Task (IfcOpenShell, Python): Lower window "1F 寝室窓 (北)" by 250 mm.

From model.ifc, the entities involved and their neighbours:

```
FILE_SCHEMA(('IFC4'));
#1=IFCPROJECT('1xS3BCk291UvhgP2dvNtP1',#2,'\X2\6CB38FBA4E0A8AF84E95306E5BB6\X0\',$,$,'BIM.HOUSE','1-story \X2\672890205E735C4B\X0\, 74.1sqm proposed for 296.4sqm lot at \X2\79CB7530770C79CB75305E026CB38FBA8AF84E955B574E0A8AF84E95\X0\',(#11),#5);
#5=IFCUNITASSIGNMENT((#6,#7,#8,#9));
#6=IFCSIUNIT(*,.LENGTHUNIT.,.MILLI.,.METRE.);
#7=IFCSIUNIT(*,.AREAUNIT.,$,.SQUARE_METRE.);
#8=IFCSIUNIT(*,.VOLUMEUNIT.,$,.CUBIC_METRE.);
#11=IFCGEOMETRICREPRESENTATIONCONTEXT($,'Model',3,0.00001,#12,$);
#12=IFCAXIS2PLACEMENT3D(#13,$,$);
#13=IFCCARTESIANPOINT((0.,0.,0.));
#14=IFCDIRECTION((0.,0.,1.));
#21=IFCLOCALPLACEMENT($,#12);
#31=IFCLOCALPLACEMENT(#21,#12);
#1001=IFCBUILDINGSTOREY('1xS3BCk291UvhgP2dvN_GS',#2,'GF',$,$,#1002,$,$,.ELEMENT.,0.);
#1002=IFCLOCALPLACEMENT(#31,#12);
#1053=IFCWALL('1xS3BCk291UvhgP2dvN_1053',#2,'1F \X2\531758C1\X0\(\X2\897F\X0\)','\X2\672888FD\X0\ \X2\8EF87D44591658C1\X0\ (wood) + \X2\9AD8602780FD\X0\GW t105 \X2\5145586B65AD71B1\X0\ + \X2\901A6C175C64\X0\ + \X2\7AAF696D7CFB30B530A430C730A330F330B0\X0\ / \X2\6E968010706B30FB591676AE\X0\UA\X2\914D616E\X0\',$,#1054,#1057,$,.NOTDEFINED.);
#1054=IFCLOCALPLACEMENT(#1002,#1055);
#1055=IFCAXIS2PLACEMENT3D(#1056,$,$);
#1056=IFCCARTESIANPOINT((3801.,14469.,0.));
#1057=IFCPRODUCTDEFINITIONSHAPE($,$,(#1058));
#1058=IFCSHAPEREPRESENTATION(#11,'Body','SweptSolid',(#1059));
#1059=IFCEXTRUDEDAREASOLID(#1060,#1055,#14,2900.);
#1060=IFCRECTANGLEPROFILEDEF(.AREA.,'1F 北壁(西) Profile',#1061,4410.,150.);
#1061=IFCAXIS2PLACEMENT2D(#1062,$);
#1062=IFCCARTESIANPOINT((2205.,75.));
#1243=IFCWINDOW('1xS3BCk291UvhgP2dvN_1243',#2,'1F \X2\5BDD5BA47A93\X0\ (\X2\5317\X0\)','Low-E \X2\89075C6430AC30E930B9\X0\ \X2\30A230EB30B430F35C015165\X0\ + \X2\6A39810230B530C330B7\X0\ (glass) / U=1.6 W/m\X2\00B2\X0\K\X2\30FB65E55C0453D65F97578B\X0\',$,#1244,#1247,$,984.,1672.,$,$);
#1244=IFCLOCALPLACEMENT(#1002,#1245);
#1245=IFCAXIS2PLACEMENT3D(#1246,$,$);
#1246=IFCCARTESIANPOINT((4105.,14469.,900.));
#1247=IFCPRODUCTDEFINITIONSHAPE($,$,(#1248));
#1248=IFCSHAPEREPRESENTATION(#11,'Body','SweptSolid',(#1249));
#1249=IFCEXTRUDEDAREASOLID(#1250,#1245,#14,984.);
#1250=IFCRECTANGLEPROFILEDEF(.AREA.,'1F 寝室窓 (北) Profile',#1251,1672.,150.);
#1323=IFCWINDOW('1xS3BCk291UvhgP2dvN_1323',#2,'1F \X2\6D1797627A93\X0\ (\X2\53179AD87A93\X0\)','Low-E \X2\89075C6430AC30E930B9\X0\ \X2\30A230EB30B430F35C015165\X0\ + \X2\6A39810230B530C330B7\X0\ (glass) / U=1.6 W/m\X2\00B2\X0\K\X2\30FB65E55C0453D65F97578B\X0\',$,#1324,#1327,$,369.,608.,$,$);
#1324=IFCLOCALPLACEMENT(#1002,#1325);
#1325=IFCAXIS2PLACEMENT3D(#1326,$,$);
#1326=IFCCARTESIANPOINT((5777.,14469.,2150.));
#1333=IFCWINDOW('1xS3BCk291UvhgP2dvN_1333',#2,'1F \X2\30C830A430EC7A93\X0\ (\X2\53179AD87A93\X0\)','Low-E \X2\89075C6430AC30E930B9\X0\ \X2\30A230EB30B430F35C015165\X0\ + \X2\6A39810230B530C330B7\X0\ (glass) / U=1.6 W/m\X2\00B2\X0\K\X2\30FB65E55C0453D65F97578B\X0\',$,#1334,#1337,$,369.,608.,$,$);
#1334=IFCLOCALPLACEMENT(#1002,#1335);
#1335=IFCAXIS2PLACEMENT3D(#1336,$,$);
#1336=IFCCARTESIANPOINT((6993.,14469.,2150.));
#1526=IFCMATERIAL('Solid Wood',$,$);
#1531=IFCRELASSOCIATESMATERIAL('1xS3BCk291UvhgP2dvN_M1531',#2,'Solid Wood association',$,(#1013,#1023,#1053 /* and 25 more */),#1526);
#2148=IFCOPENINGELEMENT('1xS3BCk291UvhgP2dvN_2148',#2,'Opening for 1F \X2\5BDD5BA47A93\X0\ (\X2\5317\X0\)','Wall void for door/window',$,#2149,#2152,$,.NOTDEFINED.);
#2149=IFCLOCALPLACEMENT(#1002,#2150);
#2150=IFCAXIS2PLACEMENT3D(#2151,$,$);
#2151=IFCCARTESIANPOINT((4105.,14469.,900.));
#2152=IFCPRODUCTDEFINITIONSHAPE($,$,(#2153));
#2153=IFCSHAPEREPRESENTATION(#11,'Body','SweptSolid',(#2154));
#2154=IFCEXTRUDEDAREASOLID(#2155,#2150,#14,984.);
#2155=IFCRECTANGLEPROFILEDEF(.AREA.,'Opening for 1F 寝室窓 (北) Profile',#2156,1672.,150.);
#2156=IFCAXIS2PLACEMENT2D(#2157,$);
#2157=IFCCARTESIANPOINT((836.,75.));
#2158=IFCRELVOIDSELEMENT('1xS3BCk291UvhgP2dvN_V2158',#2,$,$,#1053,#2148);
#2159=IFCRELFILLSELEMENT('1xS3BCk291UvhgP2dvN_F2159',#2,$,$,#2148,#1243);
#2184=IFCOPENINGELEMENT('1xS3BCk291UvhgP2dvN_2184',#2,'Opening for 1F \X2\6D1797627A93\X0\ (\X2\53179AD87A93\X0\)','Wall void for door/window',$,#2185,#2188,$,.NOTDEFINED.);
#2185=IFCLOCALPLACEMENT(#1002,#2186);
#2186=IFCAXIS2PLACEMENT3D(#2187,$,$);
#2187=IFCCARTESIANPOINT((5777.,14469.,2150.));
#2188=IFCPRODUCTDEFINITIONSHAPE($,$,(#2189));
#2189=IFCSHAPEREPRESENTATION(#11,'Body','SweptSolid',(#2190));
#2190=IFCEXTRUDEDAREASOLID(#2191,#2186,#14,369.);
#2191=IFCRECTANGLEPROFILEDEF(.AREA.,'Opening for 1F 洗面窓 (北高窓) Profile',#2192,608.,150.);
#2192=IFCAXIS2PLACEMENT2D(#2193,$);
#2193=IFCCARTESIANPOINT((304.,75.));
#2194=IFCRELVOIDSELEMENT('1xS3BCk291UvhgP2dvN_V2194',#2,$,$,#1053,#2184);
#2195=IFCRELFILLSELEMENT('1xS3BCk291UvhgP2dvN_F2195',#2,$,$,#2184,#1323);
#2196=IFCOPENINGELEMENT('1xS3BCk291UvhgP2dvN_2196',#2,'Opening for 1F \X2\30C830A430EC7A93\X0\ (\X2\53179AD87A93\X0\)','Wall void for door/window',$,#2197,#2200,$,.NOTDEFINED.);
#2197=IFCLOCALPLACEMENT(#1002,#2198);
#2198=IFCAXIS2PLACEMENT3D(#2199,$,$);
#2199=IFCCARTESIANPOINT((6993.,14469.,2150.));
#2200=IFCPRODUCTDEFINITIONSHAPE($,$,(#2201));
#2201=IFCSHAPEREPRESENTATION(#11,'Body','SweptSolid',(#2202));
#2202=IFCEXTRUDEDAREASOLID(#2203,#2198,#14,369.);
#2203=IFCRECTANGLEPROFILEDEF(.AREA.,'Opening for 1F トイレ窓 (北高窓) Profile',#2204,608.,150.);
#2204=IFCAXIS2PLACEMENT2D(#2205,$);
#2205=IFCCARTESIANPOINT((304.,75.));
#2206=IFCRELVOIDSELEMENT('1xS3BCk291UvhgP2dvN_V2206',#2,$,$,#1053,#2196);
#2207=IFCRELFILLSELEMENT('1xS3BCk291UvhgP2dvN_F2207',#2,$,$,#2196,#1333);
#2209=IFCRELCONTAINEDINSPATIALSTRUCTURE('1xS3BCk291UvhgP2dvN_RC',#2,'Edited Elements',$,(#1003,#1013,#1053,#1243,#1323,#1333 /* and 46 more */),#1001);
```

```python
import numpy as np
import ifcopenshell
import ifcopenshell.api.geometry
import ifcopenshell.util.placement
import ifcopenshell.util.unit

model = ifcopenshell.open("model.ifc")
unit_scale = ifcopenshell.util.unit.calculate_unit_scale(model)

window = model.by_guid("1xS3BCk291UvhgP2dvN_1243")
opening = window.FillsVoids[0].RelatingOpeningElement
dz = -250.0

shift = np.array([0.0, 0.0, dz])
# The window is not placed relative to its opening, so move both.
for product in (opening, window):
    matrix = ifcopenshell.util.placement.get_local_placement(product.ObjectPlacement)
    matrix[:3, 3] += shift
    ifcopenshell.api.geometry.edit_object_placement(model, product=product, matrix=matrix, is_si=False)

print(f"moved by {dz * unit_scale:+.3f} m")

model.write("model_edited.ifc")
```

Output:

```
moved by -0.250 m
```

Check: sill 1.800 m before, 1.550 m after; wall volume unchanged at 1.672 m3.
